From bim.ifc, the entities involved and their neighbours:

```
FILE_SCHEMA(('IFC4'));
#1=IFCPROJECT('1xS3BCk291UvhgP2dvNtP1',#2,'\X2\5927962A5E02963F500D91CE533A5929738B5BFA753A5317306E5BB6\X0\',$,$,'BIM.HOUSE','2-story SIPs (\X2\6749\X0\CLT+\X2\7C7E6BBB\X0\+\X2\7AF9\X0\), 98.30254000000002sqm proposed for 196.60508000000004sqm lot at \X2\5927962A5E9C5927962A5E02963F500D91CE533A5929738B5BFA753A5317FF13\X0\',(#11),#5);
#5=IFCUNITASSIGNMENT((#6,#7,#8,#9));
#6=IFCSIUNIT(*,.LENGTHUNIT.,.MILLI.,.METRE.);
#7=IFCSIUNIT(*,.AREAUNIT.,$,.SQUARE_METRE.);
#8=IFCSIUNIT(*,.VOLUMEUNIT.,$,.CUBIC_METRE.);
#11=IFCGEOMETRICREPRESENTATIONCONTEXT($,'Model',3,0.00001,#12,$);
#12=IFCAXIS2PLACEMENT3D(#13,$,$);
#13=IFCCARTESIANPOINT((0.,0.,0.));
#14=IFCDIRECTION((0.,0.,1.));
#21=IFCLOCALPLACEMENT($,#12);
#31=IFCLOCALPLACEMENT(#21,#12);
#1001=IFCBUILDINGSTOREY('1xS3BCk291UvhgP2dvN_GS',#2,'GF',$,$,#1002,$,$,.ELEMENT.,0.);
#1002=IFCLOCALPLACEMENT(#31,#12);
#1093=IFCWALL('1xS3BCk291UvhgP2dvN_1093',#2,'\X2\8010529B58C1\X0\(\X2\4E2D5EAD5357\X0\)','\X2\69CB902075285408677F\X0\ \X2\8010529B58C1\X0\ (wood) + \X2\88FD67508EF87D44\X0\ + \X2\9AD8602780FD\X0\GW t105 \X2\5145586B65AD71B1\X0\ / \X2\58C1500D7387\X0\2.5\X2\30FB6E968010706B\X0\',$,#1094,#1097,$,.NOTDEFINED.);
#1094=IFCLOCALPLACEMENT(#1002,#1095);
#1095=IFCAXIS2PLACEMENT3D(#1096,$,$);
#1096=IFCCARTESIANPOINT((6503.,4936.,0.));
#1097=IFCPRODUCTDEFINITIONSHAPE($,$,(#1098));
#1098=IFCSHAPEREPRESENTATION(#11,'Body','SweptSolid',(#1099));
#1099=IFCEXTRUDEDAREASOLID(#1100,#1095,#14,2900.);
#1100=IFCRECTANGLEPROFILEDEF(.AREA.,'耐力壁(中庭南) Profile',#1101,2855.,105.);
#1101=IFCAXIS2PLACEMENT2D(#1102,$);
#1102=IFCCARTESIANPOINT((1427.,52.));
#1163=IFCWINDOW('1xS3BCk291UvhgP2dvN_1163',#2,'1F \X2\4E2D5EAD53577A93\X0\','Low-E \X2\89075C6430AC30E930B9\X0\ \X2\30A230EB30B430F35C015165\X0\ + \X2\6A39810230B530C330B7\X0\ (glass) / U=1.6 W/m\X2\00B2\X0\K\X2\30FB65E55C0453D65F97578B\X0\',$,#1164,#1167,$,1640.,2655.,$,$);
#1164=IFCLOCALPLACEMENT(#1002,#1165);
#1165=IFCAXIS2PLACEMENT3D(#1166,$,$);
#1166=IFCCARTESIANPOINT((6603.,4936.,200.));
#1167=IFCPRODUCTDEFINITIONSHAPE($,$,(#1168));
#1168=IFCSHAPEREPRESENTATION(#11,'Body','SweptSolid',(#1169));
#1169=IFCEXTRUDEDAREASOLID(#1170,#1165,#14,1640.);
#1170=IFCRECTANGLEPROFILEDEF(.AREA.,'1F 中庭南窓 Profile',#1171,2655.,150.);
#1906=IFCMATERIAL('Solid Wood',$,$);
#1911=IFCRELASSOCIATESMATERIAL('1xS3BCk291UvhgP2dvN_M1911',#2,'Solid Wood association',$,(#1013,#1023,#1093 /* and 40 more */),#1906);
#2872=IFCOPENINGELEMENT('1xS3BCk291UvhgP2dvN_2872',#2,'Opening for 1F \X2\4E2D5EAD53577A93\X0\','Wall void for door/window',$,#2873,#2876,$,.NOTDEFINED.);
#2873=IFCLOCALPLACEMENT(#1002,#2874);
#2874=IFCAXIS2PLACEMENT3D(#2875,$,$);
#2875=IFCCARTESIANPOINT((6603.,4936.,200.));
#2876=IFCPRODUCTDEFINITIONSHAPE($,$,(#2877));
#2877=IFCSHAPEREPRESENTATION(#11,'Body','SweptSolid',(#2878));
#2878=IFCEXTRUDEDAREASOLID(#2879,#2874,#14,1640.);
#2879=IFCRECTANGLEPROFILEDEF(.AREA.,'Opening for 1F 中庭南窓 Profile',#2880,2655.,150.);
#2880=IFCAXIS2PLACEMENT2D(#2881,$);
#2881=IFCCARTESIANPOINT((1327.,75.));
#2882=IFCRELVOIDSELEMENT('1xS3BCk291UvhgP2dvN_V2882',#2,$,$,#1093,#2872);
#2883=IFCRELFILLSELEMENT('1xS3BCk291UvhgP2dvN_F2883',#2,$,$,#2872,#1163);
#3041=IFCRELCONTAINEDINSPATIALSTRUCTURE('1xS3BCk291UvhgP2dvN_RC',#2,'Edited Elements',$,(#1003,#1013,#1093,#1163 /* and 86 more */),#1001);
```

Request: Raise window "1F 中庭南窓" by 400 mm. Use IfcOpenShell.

```python
import numpy as np
import ifcopenshell
import ifcopenshell.api.geometry
import ifcopenshell.util.placement
import ifcopenshell.util.unit

model = ifcopenshell.open("bim.ifc")
unit_scale = ifcopenshell.util.unit.calculate_unit_scale(model)

window = model.by_id(1163)
opening = window.FillsVoids[0].RelatingOpeningElement
dz = 0.4 / unit_scale

shift = np.array([0.0, 0.0, dz])
# The window is not placed relative to its opening, so move both.
for product in (opening, window):
    matrix = ifcopenshell.util.placement.get_local_placement(product.ObjectPlacement)
    matrix[:3, 3] += shift
    ifcopenshell.api.geometry.edit_object_placement(model, product=product, matrix=matrix, is_si=False)

print(f"moved by {dz * unit_scale:+.3f} m")

model.write("bim-out.ifc")
```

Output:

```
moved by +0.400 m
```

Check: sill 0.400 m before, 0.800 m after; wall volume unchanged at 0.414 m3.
